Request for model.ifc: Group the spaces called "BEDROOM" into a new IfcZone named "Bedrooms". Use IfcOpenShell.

First a look at what the model holds.

```python
import ifcopenshell

model = ifcopenshell.open("model.ifc")
print(model.schema)
seen = {}
for space in model.by_type("IfcSpace"):
    seen[space.LongName] = seen.get(space.LongName, 0) + 1
for name, count in sorted(seen.items(), key=str):
    print(count, "x", name)
print("zones:", [z.Name for z in model.by_type("IfcZone")][:20])
```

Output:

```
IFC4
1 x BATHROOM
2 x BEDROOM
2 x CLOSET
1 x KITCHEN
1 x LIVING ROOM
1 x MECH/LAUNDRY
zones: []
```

```python
import ifcopenshell
import ifcopenshell.api.group
import ifcopenshell.api.root

model = ifcopenshell.open("model.ifc")

names = {"BEDROOM"}
spaces = [s for s in model.by_type("IfcSpace") if s.LongName in names]

zone = ifcopenshell.api.root.create_entity(model, ifc_class="IfcZone", name="Bedrooms")
ifcopenshell.api.group.assign_group(model, products=spaces, group=zone)
print(len(spaces), "spaces in", zone.Name)

model.write("model_v2.ifc")
```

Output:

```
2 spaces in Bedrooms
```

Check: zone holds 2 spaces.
